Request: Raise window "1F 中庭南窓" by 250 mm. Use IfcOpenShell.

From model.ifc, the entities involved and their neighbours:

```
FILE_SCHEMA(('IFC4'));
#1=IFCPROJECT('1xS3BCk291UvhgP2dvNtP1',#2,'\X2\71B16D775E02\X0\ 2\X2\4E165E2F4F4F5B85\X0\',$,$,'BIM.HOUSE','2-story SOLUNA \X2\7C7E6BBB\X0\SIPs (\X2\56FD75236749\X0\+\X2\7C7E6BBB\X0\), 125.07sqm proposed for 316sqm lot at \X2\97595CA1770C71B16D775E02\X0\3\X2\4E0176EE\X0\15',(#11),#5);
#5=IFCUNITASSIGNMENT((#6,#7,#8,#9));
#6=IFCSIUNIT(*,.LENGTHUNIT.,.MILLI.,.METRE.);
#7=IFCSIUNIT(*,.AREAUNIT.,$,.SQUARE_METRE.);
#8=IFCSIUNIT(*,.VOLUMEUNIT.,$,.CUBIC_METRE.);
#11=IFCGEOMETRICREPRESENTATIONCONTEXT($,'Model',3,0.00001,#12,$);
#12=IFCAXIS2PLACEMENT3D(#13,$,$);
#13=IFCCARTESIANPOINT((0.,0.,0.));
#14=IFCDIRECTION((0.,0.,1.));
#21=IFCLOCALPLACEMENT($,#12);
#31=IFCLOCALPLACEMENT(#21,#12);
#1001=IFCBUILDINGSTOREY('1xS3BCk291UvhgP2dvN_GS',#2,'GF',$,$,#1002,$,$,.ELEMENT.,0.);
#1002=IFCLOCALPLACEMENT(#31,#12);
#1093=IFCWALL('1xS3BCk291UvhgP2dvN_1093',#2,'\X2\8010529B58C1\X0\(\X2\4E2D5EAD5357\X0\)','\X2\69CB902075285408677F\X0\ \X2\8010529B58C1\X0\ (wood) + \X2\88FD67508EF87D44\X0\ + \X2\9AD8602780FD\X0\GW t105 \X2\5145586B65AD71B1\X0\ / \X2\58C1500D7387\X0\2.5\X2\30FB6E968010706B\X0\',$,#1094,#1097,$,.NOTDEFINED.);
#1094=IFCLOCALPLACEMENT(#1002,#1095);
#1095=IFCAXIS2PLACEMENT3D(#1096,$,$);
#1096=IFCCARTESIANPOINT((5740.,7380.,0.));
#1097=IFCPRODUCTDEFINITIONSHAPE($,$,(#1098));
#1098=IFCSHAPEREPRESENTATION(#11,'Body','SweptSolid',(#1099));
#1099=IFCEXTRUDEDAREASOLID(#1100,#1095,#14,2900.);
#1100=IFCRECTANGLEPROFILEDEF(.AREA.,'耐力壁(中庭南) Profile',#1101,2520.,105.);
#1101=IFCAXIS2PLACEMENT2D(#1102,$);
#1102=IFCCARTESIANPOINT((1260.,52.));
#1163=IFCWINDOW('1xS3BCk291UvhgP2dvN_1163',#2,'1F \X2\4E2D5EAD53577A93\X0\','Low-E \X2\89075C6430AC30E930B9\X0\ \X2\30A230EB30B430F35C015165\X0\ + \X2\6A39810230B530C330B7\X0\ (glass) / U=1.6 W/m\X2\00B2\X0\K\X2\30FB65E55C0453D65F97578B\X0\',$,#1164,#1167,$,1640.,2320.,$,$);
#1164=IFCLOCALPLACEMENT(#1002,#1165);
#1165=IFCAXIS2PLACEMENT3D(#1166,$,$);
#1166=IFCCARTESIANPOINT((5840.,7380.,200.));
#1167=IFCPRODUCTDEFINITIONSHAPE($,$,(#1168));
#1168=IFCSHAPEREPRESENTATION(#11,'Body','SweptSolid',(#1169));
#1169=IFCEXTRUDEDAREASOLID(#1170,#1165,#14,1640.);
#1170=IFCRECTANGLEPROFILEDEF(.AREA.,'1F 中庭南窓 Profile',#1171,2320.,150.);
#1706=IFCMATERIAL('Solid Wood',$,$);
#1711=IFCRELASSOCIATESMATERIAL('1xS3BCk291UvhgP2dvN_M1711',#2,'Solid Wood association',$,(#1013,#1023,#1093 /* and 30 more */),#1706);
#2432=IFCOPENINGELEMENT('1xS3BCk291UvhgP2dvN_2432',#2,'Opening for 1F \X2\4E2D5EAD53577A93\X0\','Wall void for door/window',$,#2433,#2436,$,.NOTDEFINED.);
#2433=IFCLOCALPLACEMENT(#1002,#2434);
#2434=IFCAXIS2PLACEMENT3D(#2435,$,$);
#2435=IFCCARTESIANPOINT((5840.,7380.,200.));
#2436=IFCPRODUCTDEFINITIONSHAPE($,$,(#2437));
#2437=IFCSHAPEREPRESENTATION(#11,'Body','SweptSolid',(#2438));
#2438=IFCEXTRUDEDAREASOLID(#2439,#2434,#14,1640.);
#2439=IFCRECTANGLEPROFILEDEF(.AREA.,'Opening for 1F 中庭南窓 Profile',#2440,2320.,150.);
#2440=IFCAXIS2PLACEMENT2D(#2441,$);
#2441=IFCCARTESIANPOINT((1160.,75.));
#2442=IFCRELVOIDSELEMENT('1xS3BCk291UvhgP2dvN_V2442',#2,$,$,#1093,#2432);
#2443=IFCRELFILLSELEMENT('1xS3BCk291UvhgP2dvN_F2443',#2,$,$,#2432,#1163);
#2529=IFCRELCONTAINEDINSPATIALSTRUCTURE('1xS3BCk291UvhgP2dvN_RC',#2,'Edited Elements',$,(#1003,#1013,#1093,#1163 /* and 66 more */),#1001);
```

```python
import numpy as np
import ifcopenshell
import ifcopenshell.api.geometry
import ifcopenshell.util.placement
import ifcopenshell.util.unit

model = ifcopenshell.open("model.ifc")
unit_scale = ifcopenshell.util.unit.calculate_unit_scale(model)

window = model.by_guid("1xS3BCk291UvhgP2dvN_1163")
opening = window.FillsVoids[0].RelatingOpeningElement
dz = 250.0

shift = np.array([0.0, 0.0, dz])
# The window is not placed relative to its opening, so move both.
for product in (opening, window):
    matrix = ifcopenshell.util.placement.get_local_placement(product.ObjectPlacement)
    matrix[:3, 3] += shift
    ifcopenshell.api.geometry.edit_object_placement(model, product=product, matrix=matrix, is_si=False)

print(f"moved by {dz * unit_scale:+.3f} m")

model.write("model_rev.ifc")
```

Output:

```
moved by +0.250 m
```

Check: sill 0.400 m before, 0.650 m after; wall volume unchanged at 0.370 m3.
